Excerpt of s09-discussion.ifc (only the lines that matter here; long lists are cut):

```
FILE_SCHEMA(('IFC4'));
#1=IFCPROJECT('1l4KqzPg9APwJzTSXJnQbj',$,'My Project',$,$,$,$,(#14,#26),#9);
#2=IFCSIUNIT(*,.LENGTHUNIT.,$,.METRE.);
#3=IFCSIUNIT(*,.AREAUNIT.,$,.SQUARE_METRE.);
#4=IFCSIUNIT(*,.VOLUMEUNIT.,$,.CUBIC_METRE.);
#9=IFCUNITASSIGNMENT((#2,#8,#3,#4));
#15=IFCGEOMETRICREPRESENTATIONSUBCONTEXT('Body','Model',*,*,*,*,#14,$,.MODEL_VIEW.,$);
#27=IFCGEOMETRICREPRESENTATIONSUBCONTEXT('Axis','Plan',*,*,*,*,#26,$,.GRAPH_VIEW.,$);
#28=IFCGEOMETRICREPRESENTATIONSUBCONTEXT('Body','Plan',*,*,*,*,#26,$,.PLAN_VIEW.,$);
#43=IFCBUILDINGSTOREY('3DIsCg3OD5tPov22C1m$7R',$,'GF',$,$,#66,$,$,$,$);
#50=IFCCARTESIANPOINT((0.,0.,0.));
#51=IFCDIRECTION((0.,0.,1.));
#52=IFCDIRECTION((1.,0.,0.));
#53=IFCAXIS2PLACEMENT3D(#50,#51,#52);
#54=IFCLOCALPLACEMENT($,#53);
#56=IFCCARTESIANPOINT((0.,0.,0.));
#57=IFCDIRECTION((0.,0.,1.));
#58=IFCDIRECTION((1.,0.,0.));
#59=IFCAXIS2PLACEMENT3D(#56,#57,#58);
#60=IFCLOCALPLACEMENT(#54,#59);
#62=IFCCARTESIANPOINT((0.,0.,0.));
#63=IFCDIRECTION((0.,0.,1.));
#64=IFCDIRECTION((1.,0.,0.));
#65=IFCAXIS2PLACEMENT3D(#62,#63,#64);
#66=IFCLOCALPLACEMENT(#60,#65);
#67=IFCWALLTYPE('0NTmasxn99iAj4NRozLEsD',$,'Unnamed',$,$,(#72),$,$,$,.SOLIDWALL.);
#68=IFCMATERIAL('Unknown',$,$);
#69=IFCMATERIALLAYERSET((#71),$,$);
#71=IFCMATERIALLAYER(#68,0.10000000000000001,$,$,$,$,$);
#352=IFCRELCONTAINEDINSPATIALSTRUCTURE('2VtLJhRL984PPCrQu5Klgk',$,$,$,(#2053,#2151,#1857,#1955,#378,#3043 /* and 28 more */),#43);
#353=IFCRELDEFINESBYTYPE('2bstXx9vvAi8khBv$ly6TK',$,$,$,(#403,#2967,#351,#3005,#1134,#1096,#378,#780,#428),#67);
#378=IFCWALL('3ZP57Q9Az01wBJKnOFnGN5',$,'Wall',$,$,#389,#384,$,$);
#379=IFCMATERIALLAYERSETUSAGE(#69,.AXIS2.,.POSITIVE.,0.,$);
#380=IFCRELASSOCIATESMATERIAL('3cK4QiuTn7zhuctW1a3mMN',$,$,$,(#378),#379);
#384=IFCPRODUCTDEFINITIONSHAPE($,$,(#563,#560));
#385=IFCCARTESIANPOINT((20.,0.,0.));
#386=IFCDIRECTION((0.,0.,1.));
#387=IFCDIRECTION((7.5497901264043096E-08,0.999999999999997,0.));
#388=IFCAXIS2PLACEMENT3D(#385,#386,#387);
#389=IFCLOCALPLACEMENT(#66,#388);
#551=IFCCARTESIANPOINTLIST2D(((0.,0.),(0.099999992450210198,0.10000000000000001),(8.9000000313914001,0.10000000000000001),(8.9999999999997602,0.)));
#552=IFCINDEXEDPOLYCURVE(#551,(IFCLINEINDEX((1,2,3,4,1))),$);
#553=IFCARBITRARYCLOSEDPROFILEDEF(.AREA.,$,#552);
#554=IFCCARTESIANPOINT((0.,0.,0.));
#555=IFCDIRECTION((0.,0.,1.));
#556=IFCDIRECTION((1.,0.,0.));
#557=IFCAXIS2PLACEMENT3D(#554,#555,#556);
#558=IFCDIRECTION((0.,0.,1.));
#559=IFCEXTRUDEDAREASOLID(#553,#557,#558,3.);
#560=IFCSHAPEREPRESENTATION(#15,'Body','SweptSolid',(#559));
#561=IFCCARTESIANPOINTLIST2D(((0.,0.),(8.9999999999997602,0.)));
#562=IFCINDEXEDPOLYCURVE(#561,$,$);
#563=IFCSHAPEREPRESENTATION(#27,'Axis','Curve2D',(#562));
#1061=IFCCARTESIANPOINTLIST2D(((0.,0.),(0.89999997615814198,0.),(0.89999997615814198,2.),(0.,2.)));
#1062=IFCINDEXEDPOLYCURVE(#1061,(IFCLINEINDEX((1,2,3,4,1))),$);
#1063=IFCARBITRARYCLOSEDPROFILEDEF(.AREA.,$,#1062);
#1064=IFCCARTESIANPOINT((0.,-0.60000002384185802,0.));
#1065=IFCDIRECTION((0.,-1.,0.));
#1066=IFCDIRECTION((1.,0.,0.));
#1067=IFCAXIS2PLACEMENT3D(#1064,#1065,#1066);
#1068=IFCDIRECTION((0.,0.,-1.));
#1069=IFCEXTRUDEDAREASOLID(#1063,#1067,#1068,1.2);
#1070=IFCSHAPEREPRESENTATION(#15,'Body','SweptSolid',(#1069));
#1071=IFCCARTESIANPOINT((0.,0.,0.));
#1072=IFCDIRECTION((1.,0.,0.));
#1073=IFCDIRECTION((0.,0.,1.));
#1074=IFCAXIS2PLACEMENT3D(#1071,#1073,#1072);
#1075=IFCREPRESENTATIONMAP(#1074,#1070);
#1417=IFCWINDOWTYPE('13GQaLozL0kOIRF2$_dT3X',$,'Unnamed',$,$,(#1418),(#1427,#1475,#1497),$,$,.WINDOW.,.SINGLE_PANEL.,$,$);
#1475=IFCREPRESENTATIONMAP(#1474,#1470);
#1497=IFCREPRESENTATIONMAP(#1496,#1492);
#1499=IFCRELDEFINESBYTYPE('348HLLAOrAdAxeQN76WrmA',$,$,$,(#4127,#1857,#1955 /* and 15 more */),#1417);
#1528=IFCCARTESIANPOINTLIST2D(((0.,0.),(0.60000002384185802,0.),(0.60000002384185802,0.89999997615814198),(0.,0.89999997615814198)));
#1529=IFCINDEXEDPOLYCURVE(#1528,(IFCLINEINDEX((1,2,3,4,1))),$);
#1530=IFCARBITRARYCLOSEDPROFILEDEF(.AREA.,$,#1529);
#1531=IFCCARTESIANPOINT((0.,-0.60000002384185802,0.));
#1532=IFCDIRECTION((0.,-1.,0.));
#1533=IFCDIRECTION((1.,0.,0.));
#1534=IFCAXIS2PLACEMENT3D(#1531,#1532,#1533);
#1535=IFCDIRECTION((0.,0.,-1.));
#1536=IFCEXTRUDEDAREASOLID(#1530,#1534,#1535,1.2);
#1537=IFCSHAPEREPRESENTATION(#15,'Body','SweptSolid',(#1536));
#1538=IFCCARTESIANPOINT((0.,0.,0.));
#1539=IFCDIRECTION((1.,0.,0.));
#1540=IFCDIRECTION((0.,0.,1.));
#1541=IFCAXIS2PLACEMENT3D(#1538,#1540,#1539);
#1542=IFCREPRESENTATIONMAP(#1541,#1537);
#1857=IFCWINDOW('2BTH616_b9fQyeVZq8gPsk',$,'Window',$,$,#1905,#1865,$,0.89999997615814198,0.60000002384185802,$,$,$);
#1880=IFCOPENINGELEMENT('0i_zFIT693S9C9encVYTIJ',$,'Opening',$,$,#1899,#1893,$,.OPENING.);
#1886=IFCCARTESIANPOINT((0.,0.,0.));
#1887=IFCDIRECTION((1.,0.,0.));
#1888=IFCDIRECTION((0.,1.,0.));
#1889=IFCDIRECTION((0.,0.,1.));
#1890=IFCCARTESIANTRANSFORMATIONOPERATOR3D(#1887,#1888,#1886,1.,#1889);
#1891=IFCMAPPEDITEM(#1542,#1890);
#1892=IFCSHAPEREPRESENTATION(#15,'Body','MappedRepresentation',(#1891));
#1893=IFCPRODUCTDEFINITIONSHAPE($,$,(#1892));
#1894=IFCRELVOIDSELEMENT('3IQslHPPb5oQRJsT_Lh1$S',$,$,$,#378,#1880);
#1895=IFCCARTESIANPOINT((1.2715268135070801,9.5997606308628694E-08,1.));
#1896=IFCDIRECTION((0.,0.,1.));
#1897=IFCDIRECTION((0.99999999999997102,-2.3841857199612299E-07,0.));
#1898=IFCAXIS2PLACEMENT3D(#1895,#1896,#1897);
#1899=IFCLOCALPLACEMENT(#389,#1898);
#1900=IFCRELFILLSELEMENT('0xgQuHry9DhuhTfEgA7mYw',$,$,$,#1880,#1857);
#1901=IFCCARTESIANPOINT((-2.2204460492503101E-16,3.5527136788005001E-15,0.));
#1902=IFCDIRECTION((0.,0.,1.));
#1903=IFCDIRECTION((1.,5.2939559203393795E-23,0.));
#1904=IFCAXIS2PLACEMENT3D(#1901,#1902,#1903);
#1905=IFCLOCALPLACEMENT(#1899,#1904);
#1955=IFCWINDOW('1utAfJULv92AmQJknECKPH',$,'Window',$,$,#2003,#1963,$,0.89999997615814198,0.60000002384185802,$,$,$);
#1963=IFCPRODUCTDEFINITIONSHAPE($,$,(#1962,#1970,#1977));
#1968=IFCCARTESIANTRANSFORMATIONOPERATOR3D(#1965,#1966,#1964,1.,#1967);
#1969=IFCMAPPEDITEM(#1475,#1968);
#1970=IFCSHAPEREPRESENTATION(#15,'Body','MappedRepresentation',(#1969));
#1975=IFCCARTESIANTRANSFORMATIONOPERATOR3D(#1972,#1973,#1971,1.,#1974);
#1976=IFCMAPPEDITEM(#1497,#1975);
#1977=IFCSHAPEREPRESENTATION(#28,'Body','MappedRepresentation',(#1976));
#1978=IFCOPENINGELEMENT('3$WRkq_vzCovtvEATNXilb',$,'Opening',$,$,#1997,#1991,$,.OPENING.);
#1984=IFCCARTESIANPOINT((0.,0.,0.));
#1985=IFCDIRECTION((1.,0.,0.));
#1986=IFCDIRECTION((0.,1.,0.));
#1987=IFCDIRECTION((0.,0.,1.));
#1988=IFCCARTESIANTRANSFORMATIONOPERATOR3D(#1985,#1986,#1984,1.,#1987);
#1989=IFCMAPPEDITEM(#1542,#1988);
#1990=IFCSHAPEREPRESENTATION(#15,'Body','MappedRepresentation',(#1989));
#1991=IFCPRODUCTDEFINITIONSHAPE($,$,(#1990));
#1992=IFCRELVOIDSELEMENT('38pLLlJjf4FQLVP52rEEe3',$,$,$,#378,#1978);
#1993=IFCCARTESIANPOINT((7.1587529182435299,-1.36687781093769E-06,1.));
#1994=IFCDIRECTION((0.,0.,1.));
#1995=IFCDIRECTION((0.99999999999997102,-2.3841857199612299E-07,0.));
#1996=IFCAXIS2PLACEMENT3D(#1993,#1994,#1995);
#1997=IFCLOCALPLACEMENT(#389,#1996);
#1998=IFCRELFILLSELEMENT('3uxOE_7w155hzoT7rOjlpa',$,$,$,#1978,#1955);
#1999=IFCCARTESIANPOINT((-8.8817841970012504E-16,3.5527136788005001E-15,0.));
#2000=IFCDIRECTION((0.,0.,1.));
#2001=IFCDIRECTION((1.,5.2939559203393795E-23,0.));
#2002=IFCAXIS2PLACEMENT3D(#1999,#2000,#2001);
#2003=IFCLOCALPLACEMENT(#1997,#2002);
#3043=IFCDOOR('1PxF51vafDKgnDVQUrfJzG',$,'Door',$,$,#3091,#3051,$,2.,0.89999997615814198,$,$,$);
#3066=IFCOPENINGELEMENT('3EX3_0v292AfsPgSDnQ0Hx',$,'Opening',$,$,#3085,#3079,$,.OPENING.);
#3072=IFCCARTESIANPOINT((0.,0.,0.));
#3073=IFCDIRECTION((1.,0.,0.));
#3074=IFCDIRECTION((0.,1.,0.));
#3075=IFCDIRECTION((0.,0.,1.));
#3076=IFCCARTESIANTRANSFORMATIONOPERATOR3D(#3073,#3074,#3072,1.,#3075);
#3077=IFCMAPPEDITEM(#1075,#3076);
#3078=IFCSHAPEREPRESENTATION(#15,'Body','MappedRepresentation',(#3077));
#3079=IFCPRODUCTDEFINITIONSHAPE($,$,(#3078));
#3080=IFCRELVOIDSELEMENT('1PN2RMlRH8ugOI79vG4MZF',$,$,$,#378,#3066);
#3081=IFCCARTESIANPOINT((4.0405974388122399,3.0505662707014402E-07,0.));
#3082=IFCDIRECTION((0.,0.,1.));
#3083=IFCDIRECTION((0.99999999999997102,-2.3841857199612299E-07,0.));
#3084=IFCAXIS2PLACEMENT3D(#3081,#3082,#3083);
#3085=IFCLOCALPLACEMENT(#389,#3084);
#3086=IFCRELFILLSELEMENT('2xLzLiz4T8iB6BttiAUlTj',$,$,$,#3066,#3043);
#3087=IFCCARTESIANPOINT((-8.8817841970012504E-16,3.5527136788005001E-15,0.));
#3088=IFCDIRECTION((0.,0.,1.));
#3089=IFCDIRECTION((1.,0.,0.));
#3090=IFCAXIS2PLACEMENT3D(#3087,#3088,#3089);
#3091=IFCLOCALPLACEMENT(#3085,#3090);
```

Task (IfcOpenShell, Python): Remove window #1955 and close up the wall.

```python
import ifcopenshell
import ifcopenshell.api.feature
import ifcopenshell.api.root
import ifcopenshell.geom
import ifcopenshell.util.shape

model = ifcopenshell.open("s09-discussion.ifc")
settings = ifcopenshell.geom.settings()


def volume(element):
    """Net volume in cubic metres, openings subtracted."""
    shape = ifcopenshell.geom.create_shape(settings, element)
    return ifcopenshell.util.shape.get_volume(shape.geometry)


window = model.by_guid("1utAfJULv92AmQJknECKPH")
opening = window.FillsVoids[0].RelatingOpeningElement
wall = opening.VoidsElements[0].RelatingBuildingElement
before = volume(wall)

ifcopenshell.api.root.remove_product(model, product=window)
ifcopenshell.api.feature.remove_feature(model, feature=opening)

after = volume(wall)

print(f"wall volume {before:.3f} -> {after:.3f} m3")

model.write("s09-discussion_rev.ifc")
```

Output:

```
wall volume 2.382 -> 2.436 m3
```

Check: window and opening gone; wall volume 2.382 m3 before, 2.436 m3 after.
